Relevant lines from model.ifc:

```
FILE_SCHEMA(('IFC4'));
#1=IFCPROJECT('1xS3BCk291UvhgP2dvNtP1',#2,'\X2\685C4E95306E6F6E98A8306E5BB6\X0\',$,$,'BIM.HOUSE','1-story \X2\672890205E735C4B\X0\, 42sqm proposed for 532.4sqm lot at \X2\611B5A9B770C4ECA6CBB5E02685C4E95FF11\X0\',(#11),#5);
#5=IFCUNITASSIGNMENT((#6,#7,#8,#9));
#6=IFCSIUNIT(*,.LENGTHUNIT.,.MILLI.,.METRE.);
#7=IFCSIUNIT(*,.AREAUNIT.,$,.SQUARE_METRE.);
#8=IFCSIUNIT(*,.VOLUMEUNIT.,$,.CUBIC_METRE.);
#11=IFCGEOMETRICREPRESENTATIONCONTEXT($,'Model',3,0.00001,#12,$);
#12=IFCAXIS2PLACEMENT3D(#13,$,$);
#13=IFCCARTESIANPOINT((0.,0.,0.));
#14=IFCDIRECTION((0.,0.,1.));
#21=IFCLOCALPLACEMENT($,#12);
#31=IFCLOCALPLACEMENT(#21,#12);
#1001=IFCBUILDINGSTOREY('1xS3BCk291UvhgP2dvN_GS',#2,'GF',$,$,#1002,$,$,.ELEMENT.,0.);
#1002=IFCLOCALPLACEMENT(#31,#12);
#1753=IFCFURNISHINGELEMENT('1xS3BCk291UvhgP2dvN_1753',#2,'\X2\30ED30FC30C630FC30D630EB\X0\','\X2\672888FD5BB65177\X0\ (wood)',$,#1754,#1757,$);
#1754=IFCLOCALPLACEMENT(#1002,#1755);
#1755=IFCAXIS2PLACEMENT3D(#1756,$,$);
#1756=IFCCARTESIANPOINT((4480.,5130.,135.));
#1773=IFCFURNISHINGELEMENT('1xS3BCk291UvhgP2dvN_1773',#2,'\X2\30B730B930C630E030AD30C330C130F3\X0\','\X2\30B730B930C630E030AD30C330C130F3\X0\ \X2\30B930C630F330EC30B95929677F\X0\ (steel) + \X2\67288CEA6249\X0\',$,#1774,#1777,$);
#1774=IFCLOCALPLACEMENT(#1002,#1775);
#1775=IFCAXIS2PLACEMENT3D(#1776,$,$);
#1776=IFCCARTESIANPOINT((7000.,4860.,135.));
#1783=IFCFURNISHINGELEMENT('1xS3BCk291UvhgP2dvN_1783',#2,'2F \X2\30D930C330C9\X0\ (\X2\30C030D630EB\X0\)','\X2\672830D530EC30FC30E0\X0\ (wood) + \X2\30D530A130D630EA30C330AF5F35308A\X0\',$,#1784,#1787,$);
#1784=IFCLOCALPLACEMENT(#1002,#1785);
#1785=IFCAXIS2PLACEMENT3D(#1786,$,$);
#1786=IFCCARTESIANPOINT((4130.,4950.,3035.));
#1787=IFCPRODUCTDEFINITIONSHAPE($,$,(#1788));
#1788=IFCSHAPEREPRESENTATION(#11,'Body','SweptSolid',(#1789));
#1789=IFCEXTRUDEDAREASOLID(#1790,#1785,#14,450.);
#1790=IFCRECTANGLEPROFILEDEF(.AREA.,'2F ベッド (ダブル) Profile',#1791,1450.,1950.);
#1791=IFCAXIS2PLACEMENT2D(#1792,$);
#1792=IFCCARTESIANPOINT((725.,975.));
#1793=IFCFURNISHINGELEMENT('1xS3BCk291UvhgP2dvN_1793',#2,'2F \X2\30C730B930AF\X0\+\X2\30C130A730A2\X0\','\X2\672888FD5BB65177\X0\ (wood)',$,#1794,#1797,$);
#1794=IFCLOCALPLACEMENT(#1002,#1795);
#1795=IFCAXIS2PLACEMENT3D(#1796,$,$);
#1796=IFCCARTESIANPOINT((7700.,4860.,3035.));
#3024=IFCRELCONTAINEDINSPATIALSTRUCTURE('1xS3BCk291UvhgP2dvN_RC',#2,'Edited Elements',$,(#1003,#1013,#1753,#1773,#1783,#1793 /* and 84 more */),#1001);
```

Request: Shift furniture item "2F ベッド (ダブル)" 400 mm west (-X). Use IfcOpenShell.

```python
import ifcopenshell
import ifcopenshell.api.geometry
import ifcopenshell.util.placement
import ifcopenshell.util.unit

model = ifcopenshell.open("model.ifc")
unit_scale = ifcopenshell.util.unit.calculate_unit_scale(model)

item = model.by_guid("1xS3BCk291UvhgP2dvN_1783")
matrix = ifcopenshell.util.placement.get_local_placement(item.ObjectPlacement)
matrix[0, 3] -= 0.4 / unit_scale
ifcopenshell.api.geometry.edit_object_placement(model, product=item, matrix=matrix, is_si=False)

print(ifcopenshell.util.placement.get_local_placement(item.ObjectPlacement).round(3) + 0.0)

model.write("model_v2.ifc")
```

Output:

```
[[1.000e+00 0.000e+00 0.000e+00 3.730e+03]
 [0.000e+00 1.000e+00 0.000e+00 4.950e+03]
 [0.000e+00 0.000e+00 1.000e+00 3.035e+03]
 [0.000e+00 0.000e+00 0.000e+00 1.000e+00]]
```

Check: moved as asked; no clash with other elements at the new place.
